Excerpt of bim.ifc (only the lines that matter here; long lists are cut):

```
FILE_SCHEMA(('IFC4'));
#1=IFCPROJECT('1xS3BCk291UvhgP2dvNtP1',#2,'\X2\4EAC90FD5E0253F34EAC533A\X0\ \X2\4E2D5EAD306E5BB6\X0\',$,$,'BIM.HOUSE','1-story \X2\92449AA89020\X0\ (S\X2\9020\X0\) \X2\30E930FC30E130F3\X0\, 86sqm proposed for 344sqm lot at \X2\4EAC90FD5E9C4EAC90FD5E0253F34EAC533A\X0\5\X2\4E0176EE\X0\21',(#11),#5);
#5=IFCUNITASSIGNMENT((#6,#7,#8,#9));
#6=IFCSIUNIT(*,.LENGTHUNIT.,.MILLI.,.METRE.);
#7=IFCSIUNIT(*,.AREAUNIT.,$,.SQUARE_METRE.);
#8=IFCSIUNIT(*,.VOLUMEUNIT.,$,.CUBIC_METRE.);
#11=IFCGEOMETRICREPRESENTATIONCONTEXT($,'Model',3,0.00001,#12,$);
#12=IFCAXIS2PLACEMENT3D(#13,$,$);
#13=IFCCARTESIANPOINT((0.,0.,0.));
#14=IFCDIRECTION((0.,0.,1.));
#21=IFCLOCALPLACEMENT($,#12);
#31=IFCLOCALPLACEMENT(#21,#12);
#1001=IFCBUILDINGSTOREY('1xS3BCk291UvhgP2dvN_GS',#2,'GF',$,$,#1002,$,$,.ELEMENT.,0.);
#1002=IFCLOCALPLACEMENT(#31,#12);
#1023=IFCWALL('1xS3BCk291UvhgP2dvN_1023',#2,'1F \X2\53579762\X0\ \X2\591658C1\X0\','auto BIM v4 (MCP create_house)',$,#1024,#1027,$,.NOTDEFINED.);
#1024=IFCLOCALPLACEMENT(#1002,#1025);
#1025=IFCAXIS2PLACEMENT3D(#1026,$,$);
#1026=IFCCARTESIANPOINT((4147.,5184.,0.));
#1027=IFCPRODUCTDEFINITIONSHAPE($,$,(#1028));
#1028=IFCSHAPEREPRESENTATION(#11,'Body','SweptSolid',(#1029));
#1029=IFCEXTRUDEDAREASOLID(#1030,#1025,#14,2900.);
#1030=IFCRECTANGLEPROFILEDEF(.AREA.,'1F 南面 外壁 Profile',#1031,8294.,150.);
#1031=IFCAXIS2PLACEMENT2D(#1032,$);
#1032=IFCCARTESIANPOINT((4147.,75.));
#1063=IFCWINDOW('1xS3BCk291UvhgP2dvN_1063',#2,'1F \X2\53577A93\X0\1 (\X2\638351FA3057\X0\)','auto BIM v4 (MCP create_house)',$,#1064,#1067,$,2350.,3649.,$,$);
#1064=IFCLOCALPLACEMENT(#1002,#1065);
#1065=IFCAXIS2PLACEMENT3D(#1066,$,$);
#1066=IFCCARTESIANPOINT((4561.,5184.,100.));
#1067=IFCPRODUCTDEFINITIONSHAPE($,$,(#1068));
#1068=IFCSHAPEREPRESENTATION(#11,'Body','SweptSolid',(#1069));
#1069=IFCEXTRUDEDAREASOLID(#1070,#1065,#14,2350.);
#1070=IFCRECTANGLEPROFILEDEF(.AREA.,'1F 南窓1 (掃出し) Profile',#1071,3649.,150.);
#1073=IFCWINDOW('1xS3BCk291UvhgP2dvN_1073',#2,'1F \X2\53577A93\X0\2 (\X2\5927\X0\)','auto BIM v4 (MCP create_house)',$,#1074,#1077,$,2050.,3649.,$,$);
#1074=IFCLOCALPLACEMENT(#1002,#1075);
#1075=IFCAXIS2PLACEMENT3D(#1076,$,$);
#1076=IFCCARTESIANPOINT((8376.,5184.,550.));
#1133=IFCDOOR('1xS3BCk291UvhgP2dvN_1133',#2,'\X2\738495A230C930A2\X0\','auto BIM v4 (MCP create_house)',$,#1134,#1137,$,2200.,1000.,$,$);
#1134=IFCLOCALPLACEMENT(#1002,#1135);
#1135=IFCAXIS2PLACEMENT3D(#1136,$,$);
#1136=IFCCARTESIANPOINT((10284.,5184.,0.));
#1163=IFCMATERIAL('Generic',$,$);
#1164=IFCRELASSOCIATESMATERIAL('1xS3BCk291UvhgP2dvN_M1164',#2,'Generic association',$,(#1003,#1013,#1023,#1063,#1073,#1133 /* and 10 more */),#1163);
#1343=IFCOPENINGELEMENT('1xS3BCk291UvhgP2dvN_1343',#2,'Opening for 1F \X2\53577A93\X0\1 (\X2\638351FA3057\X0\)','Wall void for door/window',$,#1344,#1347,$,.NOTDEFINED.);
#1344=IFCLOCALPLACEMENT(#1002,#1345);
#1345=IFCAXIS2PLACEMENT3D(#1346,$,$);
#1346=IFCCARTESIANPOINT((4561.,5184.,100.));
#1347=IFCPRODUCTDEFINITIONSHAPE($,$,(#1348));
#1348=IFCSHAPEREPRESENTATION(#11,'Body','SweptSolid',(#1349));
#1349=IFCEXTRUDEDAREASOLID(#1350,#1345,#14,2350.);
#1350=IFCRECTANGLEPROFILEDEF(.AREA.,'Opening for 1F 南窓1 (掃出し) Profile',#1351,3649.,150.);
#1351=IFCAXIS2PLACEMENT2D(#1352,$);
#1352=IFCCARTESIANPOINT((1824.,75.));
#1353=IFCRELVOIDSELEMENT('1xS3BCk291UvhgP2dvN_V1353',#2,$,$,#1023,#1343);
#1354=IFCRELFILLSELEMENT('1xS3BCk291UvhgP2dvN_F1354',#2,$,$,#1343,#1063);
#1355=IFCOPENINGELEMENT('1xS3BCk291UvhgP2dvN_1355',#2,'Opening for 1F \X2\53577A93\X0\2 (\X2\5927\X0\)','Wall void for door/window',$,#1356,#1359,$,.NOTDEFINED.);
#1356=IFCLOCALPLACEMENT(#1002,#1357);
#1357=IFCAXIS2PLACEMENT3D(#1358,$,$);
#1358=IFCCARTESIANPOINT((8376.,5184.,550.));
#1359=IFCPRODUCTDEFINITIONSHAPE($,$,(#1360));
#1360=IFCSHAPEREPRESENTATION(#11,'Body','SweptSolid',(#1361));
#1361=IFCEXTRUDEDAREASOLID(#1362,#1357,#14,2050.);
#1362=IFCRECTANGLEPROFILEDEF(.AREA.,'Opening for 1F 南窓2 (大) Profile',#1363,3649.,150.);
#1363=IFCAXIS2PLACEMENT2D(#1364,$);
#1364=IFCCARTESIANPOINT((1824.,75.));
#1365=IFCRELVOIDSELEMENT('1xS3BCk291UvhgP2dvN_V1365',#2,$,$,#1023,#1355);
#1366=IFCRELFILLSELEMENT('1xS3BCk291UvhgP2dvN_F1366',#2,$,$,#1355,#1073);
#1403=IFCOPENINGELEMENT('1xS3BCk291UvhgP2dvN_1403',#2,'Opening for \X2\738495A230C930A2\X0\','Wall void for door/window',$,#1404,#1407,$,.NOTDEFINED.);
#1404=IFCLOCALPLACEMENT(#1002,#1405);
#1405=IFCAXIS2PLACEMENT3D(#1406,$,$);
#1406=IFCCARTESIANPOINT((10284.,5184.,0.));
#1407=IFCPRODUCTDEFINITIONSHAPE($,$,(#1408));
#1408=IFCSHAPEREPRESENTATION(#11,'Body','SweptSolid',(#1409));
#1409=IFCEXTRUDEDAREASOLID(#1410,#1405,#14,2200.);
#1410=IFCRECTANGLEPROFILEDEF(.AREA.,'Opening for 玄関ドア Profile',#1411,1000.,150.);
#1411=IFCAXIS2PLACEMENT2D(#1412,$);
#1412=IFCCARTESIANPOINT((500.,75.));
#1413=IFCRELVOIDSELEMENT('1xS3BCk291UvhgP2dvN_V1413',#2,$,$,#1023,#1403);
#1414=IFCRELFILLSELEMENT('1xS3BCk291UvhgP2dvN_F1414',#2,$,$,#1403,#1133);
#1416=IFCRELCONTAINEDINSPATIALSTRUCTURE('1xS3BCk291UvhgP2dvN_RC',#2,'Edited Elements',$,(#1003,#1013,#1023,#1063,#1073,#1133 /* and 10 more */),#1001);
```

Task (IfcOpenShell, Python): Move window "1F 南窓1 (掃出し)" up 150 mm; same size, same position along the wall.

```python
import numpy as np
import ifcopenshell
import ifcopenshell.api.geometry
import ifcopenshell.util.placement
import ifcopenshell.util.unit

model = ifcopenshell.open("bim.ifc")
unit_scale = ifcopenshell.util.unit.calculate_unit_scale(model)

window = model.by_guid("1xS3BCk291UvhgP2dvN_1063")
opening = window.FillsVoids[0].RelatingOpeningElement
dz = 150.0

shift = np.array([0.0, 0.0, dz])
# The window is not placed relative to its opening, so move both.
for product in (opening, window):
    matrix = ifcopenshell.util.placement.get_local_placement(product.ObjectPlacement)
    matrix[:3, 3] += shift
    ifcopenshell.api.geometry.edit_object_placement(model, product=product, matrix=matrix, is_si=False)

print(f"moved by {dz * unit_scale:+.3f} m")

model.write("bim_v2.ifc")
```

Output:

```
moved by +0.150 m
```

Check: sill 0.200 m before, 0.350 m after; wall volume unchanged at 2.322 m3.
